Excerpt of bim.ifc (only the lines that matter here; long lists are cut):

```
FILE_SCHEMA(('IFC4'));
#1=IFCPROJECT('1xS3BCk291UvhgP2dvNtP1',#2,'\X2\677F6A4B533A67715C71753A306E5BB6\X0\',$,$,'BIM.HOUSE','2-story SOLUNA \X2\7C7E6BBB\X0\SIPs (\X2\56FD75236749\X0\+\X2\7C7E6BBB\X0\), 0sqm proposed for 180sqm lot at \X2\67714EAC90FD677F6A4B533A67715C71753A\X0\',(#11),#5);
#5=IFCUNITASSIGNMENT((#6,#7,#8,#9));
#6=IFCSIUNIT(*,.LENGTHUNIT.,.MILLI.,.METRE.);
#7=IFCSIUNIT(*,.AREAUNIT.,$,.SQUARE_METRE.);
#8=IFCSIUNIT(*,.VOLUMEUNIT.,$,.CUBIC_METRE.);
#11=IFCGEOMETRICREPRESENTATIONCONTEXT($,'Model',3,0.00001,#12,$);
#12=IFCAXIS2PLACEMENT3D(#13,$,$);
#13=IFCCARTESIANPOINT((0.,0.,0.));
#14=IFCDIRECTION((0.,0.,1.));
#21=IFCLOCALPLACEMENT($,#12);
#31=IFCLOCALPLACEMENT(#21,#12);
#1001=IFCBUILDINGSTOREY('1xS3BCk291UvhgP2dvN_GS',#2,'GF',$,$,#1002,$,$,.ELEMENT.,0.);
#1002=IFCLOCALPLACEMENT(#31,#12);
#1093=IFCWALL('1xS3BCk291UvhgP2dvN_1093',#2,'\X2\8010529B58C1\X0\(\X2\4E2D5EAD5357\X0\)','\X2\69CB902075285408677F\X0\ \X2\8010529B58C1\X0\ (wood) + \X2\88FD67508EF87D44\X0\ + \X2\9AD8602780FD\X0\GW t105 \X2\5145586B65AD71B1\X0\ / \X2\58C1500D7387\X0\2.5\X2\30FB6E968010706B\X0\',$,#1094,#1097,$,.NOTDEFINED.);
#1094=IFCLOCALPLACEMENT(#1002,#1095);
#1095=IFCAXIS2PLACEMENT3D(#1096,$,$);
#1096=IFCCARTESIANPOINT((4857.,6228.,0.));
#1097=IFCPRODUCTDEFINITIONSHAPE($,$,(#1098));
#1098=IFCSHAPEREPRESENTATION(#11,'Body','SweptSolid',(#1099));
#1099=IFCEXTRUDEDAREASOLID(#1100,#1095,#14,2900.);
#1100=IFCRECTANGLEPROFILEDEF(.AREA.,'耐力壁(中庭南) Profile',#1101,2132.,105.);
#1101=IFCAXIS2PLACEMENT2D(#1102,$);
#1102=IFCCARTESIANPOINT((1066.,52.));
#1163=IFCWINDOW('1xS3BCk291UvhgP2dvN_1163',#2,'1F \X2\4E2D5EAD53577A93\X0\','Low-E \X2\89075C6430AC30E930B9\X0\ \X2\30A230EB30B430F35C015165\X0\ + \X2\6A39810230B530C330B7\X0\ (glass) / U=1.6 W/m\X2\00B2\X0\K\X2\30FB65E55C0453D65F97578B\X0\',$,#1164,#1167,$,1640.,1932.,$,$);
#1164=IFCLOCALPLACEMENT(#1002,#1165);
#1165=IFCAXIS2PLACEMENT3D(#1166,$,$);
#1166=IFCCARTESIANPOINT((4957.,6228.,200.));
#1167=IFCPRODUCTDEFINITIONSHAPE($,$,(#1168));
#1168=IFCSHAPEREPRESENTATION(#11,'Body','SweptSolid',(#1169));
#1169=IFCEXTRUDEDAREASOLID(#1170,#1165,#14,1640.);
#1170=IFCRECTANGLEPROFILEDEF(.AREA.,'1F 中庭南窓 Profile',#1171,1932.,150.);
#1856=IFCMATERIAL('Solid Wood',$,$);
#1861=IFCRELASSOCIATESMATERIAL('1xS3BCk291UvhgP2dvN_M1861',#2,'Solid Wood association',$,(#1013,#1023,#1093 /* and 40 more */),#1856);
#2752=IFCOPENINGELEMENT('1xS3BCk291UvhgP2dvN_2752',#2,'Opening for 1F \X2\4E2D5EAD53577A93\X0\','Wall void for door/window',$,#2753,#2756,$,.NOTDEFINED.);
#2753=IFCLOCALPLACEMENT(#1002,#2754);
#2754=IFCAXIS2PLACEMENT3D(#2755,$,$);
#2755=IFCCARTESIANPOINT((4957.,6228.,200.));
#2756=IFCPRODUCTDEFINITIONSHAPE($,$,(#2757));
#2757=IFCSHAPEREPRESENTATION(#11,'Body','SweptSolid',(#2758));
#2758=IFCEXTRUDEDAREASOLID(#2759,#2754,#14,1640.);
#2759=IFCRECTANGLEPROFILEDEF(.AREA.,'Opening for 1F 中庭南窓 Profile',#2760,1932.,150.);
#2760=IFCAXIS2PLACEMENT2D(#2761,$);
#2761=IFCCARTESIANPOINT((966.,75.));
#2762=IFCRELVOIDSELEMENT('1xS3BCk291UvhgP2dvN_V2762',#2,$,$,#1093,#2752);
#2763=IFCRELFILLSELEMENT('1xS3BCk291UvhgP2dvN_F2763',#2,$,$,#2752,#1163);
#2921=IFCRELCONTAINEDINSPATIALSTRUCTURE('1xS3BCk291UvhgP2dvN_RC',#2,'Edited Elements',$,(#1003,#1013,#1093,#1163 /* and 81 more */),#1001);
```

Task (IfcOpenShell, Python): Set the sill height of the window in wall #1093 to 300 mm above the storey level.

```python
import numpy as np
import ifcopenshell
import ifcopenshell.api.geometry
import ifcopenshell.geom
import ifcopenshell.util.element
import ifcopenshell.util.placement
import ifcopenshell.util.shape
import ifcopenshell.util.unit

model = ifcopenshell.open("bim.ifc")
unit_scale = ifcopenshell.util.unit.calculate_unit_scale(model)

window = model.by_id(1163)
opening = window.FillsVoids[0].RelatingOpeningElement
storey = ifcopenshell.util.element.get_container(window, ifc_class="IfcBuildingStorey")
level = ifcopenshell.util.placement.get_local_placement(storey.ObjectPlacement)[2, 3]

# The opening's origin need not be at the sill, so measure its lowest point.
shape = ifcopenshell.geom.create_shape(ifcopenshell.geom.settings(), opening)
bottom = ifcopenshell.util.shape.get_shape_bottom_elevation(shape, shape.geometry) / unit_scale
dz = level + 0.3 / unit_scale - bottom

shift = np.array([0.0, 0.0, dz])
# The window is not placed relative to its opening, so move both.
for product in (opening, window):
    matrix = ifcopenshell.util.placement.get_local_placement(product.ObjectPlacement)
    matrix[:3, 3] += shift
    ifcopenshell.api.geometry.edit_object_placement(model, product=product, matrix=matrix, is_si=False)

print(f"moved by {dz * unit_scale:+.3f} m")

model.write("bim_rev.ifc")
```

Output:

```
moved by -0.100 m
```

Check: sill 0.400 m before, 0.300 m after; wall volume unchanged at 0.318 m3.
